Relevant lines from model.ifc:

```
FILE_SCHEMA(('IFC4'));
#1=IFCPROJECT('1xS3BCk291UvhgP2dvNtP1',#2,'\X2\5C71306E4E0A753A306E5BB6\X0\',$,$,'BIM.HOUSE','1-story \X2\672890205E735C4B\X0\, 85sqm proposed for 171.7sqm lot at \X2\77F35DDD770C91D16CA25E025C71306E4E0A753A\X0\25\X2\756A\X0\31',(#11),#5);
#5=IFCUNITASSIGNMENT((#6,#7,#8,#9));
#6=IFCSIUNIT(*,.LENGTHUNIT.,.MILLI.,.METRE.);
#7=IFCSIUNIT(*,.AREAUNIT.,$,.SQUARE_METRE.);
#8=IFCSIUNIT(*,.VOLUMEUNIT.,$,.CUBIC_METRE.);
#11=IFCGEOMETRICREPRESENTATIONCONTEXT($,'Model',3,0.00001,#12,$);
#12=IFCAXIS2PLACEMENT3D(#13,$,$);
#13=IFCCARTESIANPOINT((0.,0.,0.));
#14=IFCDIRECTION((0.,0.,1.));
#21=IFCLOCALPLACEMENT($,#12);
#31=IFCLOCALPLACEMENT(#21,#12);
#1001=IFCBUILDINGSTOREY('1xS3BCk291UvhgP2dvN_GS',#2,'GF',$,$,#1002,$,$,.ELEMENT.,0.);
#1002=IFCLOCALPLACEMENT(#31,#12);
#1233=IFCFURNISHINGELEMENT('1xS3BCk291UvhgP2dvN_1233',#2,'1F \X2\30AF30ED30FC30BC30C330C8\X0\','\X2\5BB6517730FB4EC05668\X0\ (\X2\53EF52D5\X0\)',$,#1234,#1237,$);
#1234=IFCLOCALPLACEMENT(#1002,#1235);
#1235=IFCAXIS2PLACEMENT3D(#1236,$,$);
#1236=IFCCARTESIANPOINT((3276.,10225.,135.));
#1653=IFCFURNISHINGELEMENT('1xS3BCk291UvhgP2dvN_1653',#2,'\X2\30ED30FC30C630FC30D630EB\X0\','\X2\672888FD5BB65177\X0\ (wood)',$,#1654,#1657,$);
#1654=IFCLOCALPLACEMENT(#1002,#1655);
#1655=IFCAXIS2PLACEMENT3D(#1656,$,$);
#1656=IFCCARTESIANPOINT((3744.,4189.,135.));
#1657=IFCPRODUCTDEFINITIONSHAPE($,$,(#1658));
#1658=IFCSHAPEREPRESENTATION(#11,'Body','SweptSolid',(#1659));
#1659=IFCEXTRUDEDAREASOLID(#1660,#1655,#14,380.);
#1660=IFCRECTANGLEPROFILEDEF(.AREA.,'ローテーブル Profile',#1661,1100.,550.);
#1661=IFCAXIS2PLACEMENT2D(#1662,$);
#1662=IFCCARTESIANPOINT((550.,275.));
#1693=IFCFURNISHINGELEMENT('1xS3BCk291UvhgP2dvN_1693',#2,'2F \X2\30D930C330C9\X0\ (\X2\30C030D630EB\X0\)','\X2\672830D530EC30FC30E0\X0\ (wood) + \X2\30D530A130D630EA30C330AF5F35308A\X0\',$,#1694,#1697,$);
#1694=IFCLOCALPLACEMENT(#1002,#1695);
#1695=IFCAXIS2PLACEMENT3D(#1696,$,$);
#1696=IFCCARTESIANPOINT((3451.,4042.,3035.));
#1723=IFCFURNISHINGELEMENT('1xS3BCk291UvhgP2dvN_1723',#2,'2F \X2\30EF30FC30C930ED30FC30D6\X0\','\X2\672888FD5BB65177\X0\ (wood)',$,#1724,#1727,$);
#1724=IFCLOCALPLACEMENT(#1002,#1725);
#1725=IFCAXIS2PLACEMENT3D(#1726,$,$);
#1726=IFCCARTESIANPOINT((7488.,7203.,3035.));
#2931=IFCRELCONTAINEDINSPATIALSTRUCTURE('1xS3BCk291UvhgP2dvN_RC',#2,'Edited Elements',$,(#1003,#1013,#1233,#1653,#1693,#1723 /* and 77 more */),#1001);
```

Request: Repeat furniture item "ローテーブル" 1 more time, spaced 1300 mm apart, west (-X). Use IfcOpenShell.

```python
import numpy as np
import ifcopenshell
import ifcopenshell.api.geometry
import ifcopenshell.api.root
import ifcopenshell.util.element
import ifcopenshell.util.placement
import ifcopenshell.util.unit

model = ifcopenshell.open("model.ifc")
unit_scale = ifcopenshell.util.unit.calculate_unit_scale(model)


def reuse_history(source, copy):
    """copy_class also copies each property set's owner history, people and application; keep the originals."""
    for rel in copy.IsDefinedBy:
        if rel.is_a("IfcRelDefinesByProperties") and (history := rel.RelatingPropertyDefinition.OwnerHistory):
            rel.RelatingPropertyDefinition.OwnerHistory = source.OwnerHistory
            ifcopenshell.util.element.remove_deep2(model, history)


source = model.by_guid("1xS3BCk291UvhgP2dvN_1653")
base = ifcopenshell.util.placement.get_local_placement(source.ObjectPlacement)
step = np.array([-1.0, 0.0, 0.0]) * 1.3 / unit_scale

for i in range(1, 2):
    copy = ifcopenshell.api.root.copy_class(model, product=source)
    copy.Representation = ifcopenshell.util.element.copy_deep(
        model, source.Representation, exclude=["IfcGeometricRepresentationContext", "IfcRepresentationMap"]
    )
    reuse_history(source, copy)
    matrix = base.copy()
    matrix[:3, 3] += i * step
    print("added at", matrix[:3, 3].round(3) + 0.0)
    ifcopenshell.api.geometry.edit_object_placement(model, product=copy, matrix=matrix, is_si=False)

model.write("model-out.ifc")
```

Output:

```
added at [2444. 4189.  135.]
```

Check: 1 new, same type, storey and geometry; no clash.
